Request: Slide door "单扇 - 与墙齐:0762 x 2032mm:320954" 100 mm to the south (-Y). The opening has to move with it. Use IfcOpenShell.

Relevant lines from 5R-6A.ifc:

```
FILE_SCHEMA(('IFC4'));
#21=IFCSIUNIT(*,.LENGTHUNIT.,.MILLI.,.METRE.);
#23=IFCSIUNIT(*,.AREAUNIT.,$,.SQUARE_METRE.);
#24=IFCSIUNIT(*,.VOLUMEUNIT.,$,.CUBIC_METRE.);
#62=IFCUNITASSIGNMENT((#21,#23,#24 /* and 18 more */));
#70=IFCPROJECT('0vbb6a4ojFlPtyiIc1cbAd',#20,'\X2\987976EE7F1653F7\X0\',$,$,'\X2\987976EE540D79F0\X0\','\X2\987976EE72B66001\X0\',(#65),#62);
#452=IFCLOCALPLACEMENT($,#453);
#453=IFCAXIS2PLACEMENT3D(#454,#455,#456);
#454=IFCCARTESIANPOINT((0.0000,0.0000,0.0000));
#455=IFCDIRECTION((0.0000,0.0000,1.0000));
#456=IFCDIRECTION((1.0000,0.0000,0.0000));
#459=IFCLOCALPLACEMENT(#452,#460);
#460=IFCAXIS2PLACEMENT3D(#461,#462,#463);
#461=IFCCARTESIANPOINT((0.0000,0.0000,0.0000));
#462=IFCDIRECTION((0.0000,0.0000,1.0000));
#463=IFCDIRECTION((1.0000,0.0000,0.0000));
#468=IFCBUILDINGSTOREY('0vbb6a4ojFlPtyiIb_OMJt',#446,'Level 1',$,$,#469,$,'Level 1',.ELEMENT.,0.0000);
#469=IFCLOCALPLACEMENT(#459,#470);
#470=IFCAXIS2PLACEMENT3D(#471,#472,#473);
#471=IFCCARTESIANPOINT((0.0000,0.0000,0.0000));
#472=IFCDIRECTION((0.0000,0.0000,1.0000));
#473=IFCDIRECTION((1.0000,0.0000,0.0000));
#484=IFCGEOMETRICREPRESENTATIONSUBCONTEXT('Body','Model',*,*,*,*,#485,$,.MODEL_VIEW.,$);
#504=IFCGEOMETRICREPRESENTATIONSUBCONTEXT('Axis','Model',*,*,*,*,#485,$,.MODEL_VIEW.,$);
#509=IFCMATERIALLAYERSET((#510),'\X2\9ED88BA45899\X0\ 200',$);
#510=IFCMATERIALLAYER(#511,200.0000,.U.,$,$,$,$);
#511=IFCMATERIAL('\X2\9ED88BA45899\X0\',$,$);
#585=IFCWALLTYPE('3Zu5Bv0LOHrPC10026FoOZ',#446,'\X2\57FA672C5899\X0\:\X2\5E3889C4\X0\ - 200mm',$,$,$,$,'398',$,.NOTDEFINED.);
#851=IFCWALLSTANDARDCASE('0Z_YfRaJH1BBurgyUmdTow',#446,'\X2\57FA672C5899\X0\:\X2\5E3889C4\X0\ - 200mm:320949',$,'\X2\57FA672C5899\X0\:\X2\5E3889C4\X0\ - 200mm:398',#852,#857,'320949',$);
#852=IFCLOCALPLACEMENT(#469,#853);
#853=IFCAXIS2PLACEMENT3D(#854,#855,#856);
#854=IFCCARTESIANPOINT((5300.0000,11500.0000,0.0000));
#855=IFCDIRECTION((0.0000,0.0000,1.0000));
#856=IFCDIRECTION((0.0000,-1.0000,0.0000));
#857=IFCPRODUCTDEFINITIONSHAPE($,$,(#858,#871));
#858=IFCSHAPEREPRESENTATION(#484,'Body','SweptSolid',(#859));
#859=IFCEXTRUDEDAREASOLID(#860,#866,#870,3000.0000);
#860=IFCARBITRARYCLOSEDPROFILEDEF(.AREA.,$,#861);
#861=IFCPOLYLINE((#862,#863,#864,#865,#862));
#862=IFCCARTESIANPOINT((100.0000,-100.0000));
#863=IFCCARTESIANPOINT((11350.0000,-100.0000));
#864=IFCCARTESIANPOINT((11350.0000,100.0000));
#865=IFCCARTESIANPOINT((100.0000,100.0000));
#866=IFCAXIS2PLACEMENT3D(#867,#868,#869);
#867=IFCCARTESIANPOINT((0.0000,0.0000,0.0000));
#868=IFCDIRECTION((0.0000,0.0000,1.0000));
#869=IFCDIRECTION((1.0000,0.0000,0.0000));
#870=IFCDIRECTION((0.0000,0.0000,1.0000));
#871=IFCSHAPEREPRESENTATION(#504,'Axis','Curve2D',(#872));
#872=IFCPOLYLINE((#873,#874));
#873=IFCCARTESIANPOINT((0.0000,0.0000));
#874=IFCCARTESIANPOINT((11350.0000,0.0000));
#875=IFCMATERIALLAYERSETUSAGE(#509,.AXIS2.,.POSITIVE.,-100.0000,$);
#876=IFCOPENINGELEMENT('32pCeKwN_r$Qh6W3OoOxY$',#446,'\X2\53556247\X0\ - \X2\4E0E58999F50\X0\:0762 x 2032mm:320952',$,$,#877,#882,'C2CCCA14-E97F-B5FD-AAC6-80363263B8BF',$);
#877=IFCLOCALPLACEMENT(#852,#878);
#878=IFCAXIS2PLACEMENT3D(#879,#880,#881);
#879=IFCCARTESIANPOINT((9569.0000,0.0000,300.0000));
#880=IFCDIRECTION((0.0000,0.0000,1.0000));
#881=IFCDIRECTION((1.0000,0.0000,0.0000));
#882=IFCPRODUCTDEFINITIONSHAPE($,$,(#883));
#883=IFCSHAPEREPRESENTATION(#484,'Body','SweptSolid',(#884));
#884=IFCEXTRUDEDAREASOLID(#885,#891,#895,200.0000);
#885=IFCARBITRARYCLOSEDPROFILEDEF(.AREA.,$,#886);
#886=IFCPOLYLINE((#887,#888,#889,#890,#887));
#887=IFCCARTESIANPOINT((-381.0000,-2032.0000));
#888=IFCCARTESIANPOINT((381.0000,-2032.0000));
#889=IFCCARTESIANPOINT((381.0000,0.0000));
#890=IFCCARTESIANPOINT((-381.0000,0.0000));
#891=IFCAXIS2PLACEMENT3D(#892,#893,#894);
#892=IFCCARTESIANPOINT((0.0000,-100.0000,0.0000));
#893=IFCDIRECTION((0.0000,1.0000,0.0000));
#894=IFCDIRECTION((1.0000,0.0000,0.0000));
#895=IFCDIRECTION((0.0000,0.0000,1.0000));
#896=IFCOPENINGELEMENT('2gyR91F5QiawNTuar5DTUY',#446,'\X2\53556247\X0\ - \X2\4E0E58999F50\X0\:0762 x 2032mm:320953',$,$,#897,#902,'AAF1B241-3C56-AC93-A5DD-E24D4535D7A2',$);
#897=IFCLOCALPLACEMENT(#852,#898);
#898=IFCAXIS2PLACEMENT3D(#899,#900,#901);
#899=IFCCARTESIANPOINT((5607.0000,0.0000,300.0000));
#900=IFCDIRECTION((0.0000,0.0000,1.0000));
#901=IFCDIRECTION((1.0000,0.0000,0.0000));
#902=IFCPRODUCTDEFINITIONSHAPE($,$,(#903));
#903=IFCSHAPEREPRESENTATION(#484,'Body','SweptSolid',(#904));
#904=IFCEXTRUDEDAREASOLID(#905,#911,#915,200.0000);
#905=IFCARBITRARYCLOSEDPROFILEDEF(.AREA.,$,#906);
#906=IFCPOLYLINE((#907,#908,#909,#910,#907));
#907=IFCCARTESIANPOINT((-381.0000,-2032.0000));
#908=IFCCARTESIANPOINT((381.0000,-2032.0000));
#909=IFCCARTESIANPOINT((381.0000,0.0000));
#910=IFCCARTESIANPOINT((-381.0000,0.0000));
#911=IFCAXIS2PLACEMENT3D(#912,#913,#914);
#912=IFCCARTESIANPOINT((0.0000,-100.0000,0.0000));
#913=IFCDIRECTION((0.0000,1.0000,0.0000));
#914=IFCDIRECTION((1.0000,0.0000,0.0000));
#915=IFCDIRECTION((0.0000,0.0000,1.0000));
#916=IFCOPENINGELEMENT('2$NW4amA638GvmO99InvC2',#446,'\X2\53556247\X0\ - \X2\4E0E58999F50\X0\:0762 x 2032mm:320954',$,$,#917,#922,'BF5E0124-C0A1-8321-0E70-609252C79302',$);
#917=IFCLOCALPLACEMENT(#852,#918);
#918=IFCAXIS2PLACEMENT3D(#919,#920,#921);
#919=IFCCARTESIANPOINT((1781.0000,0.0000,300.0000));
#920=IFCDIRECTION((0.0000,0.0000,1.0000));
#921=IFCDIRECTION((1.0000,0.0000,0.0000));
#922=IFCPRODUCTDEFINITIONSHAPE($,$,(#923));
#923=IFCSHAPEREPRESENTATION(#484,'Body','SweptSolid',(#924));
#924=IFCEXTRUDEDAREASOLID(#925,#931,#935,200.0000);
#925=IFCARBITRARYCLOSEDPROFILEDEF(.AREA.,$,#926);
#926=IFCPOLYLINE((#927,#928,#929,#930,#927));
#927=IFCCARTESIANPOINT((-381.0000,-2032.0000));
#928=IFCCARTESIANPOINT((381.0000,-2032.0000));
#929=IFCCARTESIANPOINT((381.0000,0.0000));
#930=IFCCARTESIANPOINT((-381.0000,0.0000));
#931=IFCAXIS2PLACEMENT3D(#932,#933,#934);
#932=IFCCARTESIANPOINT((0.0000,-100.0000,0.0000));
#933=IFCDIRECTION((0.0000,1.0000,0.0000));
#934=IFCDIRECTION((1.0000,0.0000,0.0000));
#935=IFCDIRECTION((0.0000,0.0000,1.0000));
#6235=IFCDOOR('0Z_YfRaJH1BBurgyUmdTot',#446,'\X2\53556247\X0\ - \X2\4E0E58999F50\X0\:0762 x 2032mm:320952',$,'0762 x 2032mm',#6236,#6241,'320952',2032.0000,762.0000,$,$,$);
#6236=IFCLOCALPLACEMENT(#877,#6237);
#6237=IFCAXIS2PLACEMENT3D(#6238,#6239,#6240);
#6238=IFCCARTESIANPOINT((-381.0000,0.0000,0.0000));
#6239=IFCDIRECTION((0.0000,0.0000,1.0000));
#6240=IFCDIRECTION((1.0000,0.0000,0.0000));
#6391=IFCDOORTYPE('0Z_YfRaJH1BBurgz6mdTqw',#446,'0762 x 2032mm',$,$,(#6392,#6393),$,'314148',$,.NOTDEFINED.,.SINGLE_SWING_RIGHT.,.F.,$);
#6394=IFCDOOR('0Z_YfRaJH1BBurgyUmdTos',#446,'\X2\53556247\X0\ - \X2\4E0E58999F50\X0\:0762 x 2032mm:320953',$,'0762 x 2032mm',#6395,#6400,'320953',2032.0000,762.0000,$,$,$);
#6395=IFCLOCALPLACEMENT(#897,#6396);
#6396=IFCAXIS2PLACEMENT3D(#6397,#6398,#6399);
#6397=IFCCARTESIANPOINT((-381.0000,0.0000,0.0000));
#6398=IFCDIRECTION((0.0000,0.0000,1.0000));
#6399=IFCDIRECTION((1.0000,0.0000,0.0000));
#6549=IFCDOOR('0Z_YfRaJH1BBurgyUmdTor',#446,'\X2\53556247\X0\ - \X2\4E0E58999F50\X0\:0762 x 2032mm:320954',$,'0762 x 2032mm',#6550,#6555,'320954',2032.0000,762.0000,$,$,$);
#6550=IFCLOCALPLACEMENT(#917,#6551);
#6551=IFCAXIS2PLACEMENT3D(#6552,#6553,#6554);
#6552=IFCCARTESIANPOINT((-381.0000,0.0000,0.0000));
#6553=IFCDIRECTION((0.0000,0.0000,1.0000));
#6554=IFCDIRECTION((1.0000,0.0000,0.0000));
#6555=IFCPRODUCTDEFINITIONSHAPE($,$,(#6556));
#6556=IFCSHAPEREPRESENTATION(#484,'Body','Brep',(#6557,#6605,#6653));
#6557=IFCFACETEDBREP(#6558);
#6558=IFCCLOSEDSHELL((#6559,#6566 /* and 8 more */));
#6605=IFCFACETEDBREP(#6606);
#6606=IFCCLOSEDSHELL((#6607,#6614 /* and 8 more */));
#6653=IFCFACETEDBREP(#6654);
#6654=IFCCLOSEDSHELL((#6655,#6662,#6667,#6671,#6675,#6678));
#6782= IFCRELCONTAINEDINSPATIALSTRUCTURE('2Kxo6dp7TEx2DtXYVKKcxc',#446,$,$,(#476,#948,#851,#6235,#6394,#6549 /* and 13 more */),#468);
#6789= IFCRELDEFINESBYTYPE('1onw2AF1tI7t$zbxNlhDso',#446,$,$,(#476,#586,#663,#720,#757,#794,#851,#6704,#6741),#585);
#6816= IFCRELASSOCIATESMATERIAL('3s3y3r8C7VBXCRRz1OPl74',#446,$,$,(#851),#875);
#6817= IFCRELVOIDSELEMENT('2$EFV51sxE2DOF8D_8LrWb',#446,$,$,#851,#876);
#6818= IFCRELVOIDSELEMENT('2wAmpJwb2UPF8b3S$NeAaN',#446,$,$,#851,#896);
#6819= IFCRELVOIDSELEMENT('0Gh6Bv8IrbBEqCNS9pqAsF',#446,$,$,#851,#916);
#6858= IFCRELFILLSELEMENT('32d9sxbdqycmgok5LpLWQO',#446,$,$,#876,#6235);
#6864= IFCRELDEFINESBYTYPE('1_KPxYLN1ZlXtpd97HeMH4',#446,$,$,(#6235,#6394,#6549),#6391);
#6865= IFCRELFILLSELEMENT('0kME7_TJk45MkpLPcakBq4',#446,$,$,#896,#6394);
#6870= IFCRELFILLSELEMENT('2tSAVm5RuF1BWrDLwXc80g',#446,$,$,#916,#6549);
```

```python
import ifcopenshell
import ifcopenshell.api.geometry
import ifcopenshell.util.placement

model = ifcopenshell.open("5R-6A.ifc")

door = model.by_guid("0Z_YfRaJH1BBurgyUmdTor")
opening = door.FillsVoids[0].RelatingOpeningElement
wall = opening.VoidsElements[0].RelatingBuildingElement

wall_matrix = ifcopenshell.util.placement.get_local_placement(wall.ObjectPlacement)
shift = wall_matrix[:3, 0] * 100.0
before = ifcopenshell.util.placement.get_local_placement(door.ObjectPlacement)[:3, 3].copy()

# The door is placed relative to its opening, so it follows when the opening moves.
matrix = ifcopenshell.util.placement.get_local_placement(opening.ObjectPlacement)
matrix[:3, 3] += shift
ifcopenshell.api.geometry.edit_object_placement(
    model, product=opening, matrix=matrix, is_si=False, should_transform_children=True
)

after = ifcopenshell.util.placement.get_local_placement(door.ObjectPlacement)[:3, 3]
print("door moved by", (after - before).round(3) + 0.0)

model.write("5R-6A-out.ifc")
```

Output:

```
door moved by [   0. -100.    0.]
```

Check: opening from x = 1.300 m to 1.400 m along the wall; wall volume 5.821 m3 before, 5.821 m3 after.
